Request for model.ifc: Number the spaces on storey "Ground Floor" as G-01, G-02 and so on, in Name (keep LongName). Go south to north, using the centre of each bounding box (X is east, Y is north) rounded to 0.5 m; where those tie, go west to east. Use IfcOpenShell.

First a look at what the model holds.

```python
import ifcopenshell
import ifcopenshell.util.element
import ifcopenshell.util.placement

model = ifcopenshell.open("model.ifc")
print(model.schema)
storey = next(s for s in model.by_type("IfcBuildingStorey") if s.Name == "Ground Floor")
spaces = [e for e in ifcopenshell.util.element.get_decomposition(storey) if e.is_a("IfcSpace")]
for e in sorted(spaces, key=lambda e: e.id()):
    origin = ifcopenshell.util.placement.get_local_placement(e.ObjectPlacement)[:3, 3]
    print(e.id(), e.Name, e.LongName, origin.round(2) + 0.0, sep=" | ")
```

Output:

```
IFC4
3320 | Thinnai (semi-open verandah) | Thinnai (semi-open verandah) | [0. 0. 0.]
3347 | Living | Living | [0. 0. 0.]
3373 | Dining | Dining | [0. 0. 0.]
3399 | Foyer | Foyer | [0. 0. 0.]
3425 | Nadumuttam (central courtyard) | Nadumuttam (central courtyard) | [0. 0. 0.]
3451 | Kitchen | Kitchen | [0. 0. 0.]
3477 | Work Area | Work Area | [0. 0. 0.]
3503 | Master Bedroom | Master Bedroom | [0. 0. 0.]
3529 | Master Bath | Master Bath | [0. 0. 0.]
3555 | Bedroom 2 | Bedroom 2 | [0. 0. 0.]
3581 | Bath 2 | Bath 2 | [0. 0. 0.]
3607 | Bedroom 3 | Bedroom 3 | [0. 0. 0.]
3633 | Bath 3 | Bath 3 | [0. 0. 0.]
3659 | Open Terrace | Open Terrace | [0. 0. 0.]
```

```python
import ifcopenshell
import ifcopenshell.geom
import ifcopenshell.util.element
import ifcopenshell.util.shape

model = ifcopenshell.open("model.ifc")
settings = ifcopenshell.geom.settings()
settings.set("use-world-coords", True)


def centre(element):
    shape = ifcopenshell.geom.create_shape(settings, element)
    return ifcopenshell.util.shape.get_bbox_centroid(shape.geometry)


storey = next(s for s in model.by_type("IfcBuildingStorey") if s.Name == "Ground Floor")
spaces = [e for e in ifcopenshell.util.element.get_decomposition(storey) if e.is_a("IfcSpace")]

# Insertion points can sit at a corner or the storey origin, so sort by the geometry (in metres).
centres = {e: centre(e) for e in spaces}
spaces.sort(key=lambda e: (round(centres[e][1] / 0.5), centres[e][0]))

for i, e in enumerate(spaces, start=1):
    number = f"G-{i:02d}"
    e.Name = number
    print(e.id(), number)

model.write("model-out.ifc")
```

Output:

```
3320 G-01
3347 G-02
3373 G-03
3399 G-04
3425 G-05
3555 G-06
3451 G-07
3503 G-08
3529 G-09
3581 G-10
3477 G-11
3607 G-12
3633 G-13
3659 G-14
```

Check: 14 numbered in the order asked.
